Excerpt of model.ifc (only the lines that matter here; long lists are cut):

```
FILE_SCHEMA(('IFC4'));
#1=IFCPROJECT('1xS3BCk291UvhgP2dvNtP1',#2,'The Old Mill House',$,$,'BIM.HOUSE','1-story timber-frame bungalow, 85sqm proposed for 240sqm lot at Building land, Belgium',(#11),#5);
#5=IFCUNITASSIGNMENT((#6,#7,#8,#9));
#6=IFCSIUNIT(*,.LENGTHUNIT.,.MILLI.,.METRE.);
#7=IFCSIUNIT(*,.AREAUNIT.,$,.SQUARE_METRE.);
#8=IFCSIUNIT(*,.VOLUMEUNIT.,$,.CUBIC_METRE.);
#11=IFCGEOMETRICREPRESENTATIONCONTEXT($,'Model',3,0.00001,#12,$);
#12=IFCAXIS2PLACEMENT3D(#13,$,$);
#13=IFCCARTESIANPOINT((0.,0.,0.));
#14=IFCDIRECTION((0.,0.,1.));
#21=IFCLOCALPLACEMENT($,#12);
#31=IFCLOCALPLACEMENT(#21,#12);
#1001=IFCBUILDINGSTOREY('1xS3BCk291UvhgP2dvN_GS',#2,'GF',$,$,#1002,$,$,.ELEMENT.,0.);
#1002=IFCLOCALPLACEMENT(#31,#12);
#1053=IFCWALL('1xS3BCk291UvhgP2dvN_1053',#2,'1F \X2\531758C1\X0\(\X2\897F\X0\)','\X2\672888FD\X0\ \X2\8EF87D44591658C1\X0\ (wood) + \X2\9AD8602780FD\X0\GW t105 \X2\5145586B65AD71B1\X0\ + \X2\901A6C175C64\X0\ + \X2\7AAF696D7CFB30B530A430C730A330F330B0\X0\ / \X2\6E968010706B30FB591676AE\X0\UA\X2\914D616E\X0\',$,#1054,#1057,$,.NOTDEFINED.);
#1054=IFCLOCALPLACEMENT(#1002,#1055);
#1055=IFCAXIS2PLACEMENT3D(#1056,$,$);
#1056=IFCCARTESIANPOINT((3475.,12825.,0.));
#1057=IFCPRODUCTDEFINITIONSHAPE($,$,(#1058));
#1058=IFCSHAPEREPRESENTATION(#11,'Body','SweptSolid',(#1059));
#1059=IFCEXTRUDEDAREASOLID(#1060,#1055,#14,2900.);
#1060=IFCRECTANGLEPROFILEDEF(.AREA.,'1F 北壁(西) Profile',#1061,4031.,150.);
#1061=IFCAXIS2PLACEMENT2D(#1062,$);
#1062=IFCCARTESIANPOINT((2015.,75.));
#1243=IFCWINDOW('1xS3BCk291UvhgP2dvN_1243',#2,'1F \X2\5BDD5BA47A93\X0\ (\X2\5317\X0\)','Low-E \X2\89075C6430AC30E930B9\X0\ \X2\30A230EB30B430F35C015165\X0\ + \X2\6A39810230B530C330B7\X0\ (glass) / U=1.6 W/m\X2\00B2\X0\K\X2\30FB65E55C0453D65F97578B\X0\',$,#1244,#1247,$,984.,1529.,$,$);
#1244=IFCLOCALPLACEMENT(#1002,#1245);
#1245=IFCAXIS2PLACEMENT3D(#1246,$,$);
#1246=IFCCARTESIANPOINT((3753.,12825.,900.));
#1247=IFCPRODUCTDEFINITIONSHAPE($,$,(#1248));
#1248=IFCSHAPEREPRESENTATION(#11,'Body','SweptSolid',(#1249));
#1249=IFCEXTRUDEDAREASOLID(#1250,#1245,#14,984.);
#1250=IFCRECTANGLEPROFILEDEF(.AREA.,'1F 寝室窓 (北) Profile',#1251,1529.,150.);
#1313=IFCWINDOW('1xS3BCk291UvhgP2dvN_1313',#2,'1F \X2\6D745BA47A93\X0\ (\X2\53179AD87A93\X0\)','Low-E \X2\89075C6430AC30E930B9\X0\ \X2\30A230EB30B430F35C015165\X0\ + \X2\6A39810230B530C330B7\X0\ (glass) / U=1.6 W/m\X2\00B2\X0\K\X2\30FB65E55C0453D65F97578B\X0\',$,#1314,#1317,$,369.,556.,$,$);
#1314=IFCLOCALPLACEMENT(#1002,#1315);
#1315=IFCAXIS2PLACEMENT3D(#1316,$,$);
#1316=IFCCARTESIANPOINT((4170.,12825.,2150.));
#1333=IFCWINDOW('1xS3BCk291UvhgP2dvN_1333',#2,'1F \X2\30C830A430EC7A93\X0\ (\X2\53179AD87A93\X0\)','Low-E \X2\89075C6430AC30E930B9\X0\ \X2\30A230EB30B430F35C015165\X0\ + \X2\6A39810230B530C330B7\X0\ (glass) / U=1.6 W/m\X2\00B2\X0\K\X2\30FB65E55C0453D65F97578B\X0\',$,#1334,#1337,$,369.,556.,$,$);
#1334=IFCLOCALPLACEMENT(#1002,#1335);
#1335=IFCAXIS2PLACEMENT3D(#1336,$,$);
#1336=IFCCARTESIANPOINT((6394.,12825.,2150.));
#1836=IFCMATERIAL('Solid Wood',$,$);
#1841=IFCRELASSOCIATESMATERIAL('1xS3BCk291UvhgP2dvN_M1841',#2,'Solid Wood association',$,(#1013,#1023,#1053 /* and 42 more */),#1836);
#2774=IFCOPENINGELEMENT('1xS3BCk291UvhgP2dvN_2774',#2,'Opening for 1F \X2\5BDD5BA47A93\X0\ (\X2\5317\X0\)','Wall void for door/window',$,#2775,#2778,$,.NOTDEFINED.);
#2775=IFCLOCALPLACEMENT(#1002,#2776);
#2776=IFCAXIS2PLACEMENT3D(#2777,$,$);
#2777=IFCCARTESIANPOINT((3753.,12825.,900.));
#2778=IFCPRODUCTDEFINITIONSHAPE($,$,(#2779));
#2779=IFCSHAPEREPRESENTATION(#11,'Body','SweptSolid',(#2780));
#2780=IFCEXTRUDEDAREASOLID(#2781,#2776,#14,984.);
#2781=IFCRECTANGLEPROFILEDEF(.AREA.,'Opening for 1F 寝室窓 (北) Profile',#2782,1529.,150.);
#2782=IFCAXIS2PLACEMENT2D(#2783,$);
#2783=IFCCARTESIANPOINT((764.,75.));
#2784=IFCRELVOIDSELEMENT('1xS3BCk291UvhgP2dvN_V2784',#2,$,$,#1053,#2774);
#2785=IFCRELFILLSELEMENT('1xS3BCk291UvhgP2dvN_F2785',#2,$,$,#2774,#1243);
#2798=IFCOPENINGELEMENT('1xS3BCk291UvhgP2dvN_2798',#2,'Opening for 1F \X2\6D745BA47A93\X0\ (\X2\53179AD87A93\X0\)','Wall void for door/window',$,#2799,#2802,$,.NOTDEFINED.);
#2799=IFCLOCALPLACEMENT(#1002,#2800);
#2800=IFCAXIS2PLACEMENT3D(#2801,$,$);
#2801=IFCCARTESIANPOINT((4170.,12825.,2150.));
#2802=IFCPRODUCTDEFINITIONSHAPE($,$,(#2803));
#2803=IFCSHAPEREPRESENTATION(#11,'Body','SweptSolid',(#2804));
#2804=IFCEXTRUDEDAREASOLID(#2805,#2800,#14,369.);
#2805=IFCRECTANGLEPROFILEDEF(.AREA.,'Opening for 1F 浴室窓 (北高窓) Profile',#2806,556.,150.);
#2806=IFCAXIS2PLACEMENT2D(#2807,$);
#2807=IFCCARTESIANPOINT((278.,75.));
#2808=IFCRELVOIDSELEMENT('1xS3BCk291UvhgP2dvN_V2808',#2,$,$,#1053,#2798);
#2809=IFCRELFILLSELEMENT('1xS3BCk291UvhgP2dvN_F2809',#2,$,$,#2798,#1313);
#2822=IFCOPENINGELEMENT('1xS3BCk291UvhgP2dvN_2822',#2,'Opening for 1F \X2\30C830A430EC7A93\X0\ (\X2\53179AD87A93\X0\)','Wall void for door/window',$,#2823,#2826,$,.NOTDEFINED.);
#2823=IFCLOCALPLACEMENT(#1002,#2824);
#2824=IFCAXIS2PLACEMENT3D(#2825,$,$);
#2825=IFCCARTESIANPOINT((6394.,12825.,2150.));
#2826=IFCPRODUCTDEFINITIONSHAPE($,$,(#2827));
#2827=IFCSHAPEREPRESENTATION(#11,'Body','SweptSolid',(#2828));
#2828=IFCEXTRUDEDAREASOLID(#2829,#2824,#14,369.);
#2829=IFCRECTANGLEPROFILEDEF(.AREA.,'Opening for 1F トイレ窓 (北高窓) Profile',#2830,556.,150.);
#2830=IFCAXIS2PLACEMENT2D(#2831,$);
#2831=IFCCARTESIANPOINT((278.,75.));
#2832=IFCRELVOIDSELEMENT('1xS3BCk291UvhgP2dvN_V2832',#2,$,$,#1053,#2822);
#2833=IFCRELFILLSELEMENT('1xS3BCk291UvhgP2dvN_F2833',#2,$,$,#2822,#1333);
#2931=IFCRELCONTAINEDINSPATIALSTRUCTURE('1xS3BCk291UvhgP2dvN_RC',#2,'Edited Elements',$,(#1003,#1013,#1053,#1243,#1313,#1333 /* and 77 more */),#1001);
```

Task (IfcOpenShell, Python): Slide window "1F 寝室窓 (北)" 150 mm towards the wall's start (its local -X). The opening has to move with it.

```python
import ifcopenshell
import ifcopenshell.api.geometry
import ifcopenshell.util.placement

model = ifcopenshell.open("model.ifc")

window = model.by_guid("1xS3BCk291UvhgP2dvN_1243")
opening = window.FillsVoids[0].RelatingOpeningElement
wall = opening.VoidsElements[0].RelatingBuildingElement

wall_matrix = ifcopenshell.util.placement.get_local_placement(wall.ObjectPlacement)
shift = wall_matrix[:3, 0] * -150.0
before = ifcopenshell.util.placement.get_local_placement(window.ObjectPlacement)[:3, 3].copy()

# The window is not placed relative to its opening, so move both.
for product in (opening, window):
    matrix = ifcopenshell.util.placement.get_local_placement(product.ObjectPlacement)
    matrix[:3, 3] += shift
    ifcopenshell.api.geometry.edit_object_placement(model, product=product, matrix=matrix, is_si=False)

after = ifcopenshell.util.placement.get_local_placement(window.ObjectPlacement)[:3, 3]
print("window moved by", (after - before).round(3) + 0.0)

model.write("model_v2.ifc")
```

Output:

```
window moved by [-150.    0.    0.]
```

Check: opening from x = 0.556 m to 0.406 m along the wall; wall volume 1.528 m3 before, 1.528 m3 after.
